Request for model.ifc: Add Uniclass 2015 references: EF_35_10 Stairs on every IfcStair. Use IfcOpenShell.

First a look at what the model holds.

```python
import ifcopenshell

model = ifcopenshell.open("model.ifc")
print(model.schema)
print("classifications:", [c.Name for c in model.by_type("IfcClassification")])
for ifc_class in ("IfcDoor", "IfcRoof", "IfcStair", "IfcWall", "IfcWindow"):
    print(ifc_class, len(model.by_type(ifc_class)))
```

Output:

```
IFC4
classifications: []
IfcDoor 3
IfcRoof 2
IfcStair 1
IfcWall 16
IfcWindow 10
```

```python
import ifcopenshell
import ifcopenshell.api.classification

model = ifcopenshell.open("model.ifc")

system = ifcopenshell.api.classification.add_classification(model, classification="Uniclass 2015")

codes = {
    "IfcStair": ("EF_35_10", "Stairs"),
}
for ifc_class, (code, name) in codes.items():
    products = model.by_type(ifc_class)
    ifcopenshell.api.classification.add_reference(
        model, products=products, classification=system, identification=code, name=name
    )
    print(code, len(products))

model.write("model_updated.ifc")
```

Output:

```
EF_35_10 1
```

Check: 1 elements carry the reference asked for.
